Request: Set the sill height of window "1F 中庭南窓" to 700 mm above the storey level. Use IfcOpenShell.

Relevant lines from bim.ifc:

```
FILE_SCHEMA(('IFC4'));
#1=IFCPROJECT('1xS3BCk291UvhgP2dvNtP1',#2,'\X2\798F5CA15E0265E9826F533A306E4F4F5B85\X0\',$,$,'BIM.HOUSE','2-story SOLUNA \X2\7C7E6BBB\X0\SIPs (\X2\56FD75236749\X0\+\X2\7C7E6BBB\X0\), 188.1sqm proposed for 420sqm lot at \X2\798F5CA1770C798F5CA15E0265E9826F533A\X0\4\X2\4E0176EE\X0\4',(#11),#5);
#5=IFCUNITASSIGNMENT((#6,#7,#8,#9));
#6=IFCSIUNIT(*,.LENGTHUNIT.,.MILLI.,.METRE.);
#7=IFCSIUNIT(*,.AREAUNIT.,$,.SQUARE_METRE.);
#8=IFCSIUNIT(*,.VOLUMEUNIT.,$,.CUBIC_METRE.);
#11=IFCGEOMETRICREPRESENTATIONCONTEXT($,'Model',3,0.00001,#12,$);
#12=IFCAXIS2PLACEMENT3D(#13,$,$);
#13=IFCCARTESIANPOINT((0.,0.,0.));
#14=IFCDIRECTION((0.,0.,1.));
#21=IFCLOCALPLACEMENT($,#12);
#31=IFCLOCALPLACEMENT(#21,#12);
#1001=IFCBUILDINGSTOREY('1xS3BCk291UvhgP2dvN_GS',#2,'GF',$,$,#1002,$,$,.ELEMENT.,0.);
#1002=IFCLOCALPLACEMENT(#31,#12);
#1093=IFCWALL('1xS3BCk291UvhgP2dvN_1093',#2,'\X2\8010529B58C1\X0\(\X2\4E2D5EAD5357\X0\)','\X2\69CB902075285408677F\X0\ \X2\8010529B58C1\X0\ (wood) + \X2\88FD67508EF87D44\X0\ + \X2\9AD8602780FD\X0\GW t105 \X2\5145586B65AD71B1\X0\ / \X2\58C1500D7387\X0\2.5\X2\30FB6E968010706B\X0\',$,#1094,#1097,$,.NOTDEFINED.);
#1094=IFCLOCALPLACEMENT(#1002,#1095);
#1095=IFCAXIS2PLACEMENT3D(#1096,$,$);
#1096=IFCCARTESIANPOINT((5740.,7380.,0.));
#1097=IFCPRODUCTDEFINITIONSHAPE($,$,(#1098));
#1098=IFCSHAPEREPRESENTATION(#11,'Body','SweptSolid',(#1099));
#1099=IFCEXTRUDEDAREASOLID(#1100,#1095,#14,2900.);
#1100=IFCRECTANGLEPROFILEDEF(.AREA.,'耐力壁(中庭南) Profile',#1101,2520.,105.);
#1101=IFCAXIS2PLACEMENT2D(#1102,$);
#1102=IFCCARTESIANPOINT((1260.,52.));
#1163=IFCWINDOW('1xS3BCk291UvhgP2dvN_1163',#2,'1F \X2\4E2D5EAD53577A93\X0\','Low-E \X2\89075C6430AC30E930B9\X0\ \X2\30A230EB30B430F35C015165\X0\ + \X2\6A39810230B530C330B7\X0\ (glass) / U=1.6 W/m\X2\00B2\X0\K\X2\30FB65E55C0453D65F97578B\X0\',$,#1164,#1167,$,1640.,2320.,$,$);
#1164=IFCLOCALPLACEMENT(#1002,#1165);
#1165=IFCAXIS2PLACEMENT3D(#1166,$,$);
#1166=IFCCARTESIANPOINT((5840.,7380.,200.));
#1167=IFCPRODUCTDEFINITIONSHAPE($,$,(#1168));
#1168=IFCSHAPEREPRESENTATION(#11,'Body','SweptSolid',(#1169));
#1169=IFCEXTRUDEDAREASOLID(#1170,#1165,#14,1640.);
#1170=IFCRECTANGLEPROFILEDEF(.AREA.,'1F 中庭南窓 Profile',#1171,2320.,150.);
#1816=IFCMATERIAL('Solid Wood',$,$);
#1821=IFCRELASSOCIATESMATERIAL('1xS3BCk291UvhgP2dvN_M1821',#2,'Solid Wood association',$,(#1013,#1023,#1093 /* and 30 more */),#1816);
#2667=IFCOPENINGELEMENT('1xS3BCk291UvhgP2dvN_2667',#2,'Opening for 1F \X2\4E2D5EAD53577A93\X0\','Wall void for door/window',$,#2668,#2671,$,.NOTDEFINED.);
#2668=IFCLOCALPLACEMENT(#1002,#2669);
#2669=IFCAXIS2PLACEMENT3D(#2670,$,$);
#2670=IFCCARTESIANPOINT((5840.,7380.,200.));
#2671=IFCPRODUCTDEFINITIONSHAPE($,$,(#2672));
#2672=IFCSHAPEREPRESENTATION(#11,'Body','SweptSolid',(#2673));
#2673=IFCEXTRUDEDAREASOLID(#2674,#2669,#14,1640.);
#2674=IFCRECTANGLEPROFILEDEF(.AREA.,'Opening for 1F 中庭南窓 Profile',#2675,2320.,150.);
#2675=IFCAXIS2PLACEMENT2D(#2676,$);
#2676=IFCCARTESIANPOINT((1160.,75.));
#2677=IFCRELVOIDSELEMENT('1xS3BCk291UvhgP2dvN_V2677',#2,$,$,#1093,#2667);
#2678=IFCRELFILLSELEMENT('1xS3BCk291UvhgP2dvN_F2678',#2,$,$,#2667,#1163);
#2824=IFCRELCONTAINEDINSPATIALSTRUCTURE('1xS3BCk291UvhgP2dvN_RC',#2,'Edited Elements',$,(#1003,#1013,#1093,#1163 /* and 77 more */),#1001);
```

```python
import numpy as np
import ifcopenshell
import ifcopenshell.api.geometry
import ifcopenshell.geom
import ifcopenshell.util.element
import ifcopenshell.util.placement
import ifcopenshell.util.shape
import ifcopenshell.util.unit

model = ifcopenshell.open("bim.ifc")
unit_scale = ifcopenshell.util.unit.calculate_unit_scale(model)

window = model.by_guid("1xS3BCk291UvhgP2dvN_1163")
opening = window.FillsVoids[0].RelatingOpeningElement
storey = ifcopenshell.util.element.get_container(window, ifc_class="IfcBuildingStorey")
level = ifcopenshell.util.placement.get_local_placement(storey.ObjectPlacement)[2, 3]

# The opening's origin need not be at the sill, so measure its lowest point.
shape = ifcopenshell.geom.create_shape(ifcopenshell.geom.settings(), opening)
bottom = ifcopenshell.util.shape.get_shape_bottom_elevation(shape, shape.geometry) / unit_scale
dz = level + 700.0 - bottom

shift = np.array([0.0, 0.0, dz])
# The window is not placed relative to its opening, so move both.
for product in (opening, window):
    matrix = ifcopenshell.util.placement.get_local_placement(product.ObjectPlacement)
    matrix[:3, 3] += shift
    ifcopenshell.api.geometry.edit_object_placement(model, product=product, matrix=matrix, is_si=False)

print(f"moved by {dz * unit_scale:+.3f} m")

model.write("bim-out.ifc")
```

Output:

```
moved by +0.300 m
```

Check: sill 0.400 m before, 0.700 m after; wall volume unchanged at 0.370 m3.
